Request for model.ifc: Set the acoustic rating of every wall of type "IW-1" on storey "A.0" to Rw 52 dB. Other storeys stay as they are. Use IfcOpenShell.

First a look at what the model holds.

```python
import ifcopenshell
import ifcopenshell.util.element

model = ifcopenshell.open("model.ifc")
print(model.schema)
storey = next(s for s in model.by_type("IfcBuildingStorey") if s.Name == "A.0")
walls = [e for e in ifcopenshell.util.element.get_decomposition(storey) if e.is_a("IfcWall")]
seen = {}
for e in walls:
    element_type = ifcopenshell.util.element.get_type(e)
    key = (element_type.Name if element_type != e and element_type else None, ifcopenshell.util.element.get_pset(e, "Pset_WallCommon", "AcousticRating"))
    seen[key] = seen.get(key, 0) + 1
for (name, value), count in sorted(seen.items(), key=str):
    print(count, "x", name, "|", value)
```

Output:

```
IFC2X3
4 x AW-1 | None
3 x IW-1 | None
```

```python
import ifcopenshell
import ifcopenshell.api.pset
import ifcopenshell.util.element

model = ifcopenshell.open("model.ifc")

storey = next(s for s in model.by_type("IfcBuildingStorey") if s.Name == "A.0")
walls = [e for e in ifcopenshell.util.element.get_decomposition(storey) if e.is_a("IfcWall")]

count = 0
for e in walls:
    element_type = ifcopenshell.util.element.get_type(e)
    if element_type in (None, e) or element_type.Name != "IW-1":
        continue
    # add_pset returns the element's existing set when there is one.
    pset = ifcopenshell.api.pset.add_pset(model, product=e, name="Pset_WallCommon")
    ifcopenshell.api.pset.edit_pset(model, pset=pset, properties={"AcousticRating": "Rw 52 dB"})
    count += 1

print(count, "walls updated")

model.write("model_updated.ifc")
```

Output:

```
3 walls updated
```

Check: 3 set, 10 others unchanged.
